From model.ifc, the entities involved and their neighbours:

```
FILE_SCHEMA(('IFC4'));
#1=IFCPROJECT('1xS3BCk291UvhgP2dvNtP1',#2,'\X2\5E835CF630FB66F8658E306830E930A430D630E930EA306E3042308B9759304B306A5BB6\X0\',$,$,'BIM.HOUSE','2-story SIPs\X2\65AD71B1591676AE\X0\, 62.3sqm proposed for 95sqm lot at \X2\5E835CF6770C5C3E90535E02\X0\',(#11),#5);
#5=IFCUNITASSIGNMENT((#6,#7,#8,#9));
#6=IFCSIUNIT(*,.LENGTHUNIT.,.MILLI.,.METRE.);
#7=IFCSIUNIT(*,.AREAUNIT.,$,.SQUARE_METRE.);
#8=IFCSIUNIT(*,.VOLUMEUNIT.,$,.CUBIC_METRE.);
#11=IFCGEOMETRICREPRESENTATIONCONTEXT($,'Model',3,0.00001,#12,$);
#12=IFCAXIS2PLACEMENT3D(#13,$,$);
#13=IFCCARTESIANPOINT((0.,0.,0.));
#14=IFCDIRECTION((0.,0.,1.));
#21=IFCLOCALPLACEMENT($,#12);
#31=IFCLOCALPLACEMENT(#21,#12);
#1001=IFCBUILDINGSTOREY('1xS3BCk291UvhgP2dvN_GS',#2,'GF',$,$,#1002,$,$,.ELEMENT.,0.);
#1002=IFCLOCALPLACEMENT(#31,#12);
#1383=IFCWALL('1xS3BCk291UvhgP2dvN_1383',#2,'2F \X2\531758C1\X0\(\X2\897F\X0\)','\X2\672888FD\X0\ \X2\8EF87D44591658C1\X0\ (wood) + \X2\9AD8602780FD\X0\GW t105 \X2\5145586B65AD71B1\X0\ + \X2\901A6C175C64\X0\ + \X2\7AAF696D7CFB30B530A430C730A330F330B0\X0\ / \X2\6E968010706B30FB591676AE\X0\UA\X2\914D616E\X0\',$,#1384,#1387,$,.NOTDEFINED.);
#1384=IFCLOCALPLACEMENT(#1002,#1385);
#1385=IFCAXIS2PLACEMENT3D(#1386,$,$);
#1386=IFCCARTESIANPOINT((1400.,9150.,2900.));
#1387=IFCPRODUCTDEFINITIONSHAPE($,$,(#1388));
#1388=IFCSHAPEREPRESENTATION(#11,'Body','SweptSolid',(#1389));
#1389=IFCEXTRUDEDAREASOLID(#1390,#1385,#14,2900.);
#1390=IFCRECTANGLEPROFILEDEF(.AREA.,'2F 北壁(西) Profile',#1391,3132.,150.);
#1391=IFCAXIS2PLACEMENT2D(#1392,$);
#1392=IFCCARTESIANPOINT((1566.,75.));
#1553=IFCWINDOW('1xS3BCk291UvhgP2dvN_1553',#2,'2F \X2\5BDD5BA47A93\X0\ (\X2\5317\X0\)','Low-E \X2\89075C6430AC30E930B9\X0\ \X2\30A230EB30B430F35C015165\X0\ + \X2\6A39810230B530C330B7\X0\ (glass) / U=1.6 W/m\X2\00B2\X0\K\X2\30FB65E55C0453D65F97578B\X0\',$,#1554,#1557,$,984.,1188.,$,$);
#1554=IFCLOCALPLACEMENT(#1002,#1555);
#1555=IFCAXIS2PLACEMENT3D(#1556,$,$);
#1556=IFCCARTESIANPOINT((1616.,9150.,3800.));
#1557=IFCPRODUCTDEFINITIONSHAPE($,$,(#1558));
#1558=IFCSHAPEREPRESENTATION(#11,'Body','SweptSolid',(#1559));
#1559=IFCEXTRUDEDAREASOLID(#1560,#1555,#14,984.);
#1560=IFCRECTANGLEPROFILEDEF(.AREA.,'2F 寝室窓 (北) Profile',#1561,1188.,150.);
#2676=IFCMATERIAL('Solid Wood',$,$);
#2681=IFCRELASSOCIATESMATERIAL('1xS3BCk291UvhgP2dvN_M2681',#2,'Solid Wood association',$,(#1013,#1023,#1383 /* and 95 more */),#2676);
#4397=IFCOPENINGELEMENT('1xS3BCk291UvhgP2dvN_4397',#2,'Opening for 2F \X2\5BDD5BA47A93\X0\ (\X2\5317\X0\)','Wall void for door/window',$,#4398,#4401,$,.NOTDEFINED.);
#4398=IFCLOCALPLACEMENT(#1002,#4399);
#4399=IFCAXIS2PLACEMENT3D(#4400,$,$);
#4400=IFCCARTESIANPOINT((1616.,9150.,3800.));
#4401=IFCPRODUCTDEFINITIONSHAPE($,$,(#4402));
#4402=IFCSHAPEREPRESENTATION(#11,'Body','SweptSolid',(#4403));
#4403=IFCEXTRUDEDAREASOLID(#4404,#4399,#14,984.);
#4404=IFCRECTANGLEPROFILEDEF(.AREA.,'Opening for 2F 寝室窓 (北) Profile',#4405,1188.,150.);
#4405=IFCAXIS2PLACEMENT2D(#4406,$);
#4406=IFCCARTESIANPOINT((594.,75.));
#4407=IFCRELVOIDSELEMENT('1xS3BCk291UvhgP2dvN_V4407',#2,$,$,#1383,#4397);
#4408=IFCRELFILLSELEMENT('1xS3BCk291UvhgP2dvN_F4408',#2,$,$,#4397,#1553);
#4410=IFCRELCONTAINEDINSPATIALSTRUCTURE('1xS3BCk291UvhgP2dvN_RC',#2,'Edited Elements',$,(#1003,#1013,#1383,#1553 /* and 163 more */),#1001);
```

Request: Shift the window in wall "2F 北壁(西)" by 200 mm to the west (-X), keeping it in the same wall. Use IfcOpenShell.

```python
import ifcopenshell
import ifcopenshell.api.geometry
import ifcopenshell.util.placement
import ifcopenshell.util.unit

model = ifcopenshell.open("model.ifc")
unit_scale = ifcopenshell.util.unit.calculate_unit_scale(model)

window = model.by_guid("1xS3BCk291UvhgP2dvN_1553")
opening = window.FillsVoids[0].RelatingOpeningElement
wall = opening.VoidsElements[0].RelatingBuildingElement

wall_matrix = ifcopenshell.util.placement.get_local_placement(wall.ObjectPlacement)
shift = wall_matrix[:3, 0] * -0.2 / unit_scale
before = ifcopenshell.util.placement.get_local_placement(window.ObjectPlacement)[:3, 3].copy()

# The window is not placed relative to its opening, so move both.
for product in (opening, window):
    matrix = ifcopenshell.util.placement.get_local_placement(product.ObjectPlacement)
    matrix[:3, 3] += shift
    ifcopenshell.api.geometry.edit_object_placement(model, product=product, matrix=matrix, is_si=False)

after = ifcopenshell.util.placement.get_local_placement(window.ObjectPlacement)[:3, 3]
print("window moved by", (after - before).round(3) + 0.0)

model.write("model_rev.ifc")
```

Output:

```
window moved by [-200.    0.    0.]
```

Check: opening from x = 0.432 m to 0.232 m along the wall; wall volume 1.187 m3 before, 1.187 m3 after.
